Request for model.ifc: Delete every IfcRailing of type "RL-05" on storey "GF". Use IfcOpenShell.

First a look at what the model holds.

```python
import ifcopenshell
import ifcopenshell.util.element

model = ifcopenshell.open("model.ifc")
print(model.schema)
storey = next(s for s in model.by_type("IfcBuildingStorey") if s.Name == "GF")
railings = [e for e in ifcopenshell.util.element.get_decomposition(storey) if e.is_a("IfcRailing")]
seen = {}
for e in railings:
    element_type = ifcopenshell.util.element.get_type(e)
    name = element_type.Name if element_type not in (None, e) else None
    seen[name] = seen.get(name, 0) + 1
for name, count in sorted(seen.items(), key=str):
    print(count, "x", name)
```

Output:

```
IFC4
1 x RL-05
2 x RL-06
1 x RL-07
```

```python
import ifcopenshell
import ifcopenshell.api.root
import ifcopenshell.util.element

model = ifcopenshell.open("model.ifc")

storey = next(s for s in model.by_type("IfcBuildingStorey") if s.Name == "GF")
railings = [e for e in ifcopenshell.util.element.get_decomposition(storey) if e.is_a("IfcRailing")]
targets = [e for e in railings if (t := ifcopenshell.util.element.get_type(e)) not in (None, e) and t.Name == "RL-05"]

for e in targets:
    ifcopenshell.api.root.remove_product(model, product=e)
print(len(targets), "removed")

model.write("model_rev.ifc")
```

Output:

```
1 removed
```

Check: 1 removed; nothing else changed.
